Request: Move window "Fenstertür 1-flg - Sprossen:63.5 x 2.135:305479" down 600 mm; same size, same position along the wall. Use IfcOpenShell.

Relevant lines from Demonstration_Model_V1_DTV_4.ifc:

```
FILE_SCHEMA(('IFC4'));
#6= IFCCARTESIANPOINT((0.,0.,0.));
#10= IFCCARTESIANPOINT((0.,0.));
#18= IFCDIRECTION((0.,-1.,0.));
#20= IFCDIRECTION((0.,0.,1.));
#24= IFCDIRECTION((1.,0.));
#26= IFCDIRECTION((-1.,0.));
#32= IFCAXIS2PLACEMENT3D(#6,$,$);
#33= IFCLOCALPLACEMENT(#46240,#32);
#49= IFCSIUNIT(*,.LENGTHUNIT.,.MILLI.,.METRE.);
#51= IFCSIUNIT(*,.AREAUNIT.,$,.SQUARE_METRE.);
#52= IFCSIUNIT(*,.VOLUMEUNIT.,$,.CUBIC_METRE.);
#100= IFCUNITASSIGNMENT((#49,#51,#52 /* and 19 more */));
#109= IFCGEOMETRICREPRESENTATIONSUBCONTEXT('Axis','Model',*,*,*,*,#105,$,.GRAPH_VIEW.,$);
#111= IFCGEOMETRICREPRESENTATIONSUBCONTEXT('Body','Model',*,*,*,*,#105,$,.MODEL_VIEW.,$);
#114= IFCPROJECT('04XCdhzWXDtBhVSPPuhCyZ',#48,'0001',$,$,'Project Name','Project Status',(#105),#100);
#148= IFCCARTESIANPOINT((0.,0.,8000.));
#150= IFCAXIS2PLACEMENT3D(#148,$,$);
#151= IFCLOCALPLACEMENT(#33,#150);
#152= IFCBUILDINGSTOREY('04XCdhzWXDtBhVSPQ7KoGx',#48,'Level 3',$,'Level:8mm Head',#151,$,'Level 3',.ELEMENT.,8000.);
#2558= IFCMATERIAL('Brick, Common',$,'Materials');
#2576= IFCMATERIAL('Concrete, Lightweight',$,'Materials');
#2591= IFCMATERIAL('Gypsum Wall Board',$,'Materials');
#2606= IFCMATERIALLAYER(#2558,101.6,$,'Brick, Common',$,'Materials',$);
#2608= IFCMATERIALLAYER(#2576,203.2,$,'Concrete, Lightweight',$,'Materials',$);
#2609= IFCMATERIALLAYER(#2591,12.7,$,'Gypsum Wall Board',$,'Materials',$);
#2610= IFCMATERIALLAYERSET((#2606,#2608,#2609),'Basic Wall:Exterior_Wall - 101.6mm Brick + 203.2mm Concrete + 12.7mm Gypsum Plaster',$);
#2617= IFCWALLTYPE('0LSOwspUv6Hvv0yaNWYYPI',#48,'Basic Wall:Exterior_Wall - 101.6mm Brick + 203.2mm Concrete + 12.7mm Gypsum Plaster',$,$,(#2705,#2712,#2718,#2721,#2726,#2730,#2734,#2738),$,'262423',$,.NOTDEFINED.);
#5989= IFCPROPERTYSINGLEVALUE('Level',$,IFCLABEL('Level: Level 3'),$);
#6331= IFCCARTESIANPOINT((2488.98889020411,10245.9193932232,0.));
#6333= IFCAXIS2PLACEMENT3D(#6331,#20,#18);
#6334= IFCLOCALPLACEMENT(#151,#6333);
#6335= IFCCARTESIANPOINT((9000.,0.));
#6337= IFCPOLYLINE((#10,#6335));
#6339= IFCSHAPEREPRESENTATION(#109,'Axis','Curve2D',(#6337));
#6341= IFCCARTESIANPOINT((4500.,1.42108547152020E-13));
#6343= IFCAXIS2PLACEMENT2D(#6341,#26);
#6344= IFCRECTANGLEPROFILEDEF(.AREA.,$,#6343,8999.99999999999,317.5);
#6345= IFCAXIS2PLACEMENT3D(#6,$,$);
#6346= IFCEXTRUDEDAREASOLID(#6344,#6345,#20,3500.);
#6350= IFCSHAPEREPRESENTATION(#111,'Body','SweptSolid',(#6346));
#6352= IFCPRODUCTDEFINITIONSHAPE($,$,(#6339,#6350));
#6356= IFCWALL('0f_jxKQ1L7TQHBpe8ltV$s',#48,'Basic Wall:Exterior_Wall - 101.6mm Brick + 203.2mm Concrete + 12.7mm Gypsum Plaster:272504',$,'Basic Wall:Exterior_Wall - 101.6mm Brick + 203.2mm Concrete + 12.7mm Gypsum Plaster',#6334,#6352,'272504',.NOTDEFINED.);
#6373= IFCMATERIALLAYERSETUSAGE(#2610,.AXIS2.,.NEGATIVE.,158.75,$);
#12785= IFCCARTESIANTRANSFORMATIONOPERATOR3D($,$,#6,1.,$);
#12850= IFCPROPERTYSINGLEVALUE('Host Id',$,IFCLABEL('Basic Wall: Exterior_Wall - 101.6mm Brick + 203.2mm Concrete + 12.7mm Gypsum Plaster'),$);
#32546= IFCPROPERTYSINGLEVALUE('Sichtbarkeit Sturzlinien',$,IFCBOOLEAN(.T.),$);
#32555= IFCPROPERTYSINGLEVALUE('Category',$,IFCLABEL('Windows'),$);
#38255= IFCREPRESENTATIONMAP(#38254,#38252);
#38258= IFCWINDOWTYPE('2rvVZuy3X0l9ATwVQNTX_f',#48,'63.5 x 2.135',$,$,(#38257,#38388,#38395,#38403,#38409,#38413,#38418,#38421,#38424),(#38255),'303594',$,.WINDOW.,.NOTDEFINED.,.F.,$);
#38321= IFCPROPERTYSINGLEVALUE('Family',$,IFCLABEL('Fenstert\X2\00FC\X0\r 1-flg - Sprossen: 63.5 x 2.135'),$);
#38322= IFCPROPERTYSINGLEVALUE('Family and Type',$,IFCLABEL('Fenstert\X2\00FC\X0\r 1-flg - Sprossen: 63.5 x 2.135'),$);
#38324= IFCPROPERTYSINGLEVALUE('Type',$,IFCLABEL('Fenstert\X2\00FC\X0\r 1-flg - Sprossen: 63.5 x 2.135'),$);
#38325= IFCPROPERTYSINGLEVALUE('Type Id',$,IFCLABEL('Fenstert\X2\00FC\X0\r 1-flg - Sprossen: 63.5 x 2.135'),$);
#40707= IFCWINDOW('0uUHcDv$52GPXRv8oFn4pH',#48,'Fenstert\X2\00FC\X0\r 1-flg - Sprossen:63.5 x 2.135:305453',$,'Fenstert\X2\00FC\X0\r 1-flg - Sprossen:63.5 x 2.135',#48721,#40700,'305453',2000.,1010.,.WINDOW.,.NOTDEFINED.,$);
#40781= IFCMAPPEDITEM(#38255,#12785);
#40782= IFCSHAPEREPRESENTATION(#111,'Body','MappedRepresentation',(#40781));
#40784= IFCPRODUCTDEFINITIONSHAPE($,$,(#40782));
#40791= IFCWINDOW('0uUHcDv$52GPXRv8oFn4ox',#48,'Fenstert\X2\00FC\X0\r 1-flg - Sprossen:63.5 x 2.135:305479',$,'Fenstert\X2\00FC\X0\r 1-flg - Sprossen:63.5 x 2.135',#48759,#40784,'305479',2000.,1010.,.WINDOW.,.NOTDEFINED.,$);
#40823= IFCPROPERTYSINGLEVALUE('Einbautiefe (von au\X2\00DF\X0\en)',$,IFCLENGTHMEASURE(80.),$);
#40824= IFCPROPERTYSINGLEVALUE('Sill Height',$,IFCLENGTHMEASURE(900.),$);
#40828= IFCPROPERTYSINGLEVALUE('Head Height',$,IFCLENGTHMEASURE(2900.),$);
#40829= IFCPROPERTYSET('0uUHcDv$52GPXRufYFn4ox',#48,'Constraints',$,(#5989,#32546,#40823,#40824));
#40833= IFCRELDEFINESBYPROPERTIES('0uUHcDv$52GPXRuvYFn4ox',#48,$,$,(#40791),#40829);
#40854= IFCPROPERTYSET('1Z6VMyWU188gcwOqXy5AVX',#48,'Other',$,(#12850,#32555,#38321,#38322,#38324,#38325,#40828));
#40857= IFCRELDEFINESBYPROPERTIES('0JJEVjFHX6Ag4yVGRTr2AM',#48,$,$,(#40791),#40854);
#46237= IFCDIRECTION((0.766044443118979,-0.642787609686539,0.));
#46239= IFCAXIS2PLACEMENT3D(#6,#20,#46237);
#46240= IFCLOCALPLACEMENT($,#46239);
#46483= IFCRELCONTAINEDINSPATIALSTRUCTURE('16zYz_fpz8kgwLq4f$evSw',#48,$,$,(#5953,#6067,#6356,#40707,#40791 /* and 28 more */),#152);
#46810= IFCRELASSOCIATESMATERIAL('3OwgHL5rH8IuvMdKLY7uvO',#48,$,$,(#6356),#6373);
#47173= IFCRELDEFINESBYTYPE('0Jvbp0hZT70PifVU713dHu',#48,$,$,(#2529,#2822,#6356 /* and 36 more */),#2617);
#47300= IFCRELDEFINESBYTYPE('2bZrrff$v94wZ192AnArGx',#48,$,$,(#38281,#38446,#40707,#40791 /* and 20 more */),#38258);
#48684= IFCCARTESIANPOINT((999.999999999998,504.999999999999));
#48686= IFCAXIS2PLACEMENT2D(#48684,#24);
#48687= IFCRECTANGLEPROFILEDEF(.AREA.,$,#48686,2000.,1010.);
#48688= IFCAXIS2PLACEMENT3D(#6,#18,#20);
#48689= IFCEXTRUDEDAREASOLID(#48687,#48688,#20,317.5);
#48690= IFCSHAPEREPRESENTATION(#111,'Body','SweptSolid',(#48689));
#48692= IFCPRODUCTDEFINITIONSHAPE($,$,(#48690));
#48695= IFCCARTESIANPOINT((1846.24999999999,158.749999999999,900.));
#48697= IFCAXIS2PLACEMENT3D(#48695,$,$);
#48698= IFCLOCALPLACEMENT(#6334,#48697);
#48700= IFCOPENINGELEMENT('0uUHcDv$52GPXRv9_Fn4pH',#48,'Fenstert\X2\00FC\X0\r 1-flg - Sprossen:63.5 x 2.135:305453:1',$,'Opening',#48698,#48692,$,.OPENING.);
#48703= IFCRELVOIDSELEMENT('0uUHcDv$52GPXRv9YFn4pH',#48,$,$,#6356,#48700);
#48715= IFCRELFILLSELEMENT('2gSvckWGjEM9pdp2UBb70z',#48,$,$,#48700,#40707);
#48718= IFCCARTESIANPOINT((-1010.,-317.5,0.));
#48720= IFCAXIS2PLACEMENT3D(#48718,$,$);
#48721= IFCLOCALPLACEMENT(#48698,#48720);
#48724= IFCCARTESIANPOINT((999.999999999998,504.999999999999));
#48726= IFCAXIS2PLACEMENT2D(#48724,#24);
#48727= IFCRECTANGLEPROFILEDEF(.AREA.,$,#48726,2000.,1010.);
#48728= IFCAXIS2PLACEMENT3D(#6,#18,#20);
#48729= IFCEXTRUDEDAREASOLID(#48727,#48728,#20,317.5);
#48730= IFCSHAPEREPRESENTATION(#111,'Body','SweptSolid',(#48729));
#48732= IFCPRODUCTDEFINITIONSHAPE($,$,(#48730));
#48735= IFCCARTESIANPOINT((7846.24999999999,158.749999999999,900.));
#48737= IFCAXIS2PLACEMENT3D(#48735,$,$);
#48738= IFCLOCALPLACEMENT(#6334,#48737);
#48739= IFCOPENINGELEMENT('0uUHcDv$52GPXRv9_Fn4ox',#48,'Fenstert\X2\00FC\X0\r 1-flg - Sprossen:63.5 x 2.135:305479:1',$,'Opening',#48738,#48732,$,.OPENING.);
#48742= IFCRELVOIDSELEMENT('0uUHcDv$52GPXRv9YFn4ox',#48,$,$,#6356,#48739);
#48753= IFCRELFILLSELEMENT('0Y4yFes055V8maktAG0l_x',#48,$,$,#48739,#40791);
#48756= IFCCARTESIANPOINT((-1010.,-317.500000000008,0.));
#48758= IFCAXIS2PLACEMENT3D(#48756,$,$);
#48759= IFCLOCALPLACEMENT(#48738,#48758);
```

```python
import numpy as np
import ifcopenshell
import ifcopenshell.api.geometry
import ifcopenshell.api.pset
import ifcopenshell.util.element
import ifcopenshell.util.placement
import ifcopenshell.util.unit

model = ifcopenshell.open("Demonstration_Model_V1_DTV_4.ifc")
unit_scale = ifcopenshell.util.unit.calculate_unit_scale(model)

window = model.by_guid("0uUHcDv$52GPXRv8oFn4ox")
opening = window.FillsVoids[0].RelatingOpeningElement
dz = -0.6 / unit_scale

shift = np.array([0.0, 0.0, dz])
# The window is placed relative to its opening, so it follows when the opening moves.
matrix = ifcopenshell.util.placement.get_local_placement(opening.ObjectPlacement)
matrix[:3, 3] += shift
ifcopenshell.api.geometry.edit_object_placement(
    model, product=opening, matrix=matrix, is_si=False, should_transform_children=True
)

# Keep the stored heights in step.
pset = model.by_id(ifcopenshell.util.element.get_pset(window, "Constraints", should_inherit=False)["id"])
ifcopenshell.api.pset.edit_pset(model, pset=pset, properties={
    "Sill Height": model.create_entity("IfcLengthMeasure", ifcopenshell.util.element.get_pset(window, "Constraints", "Sill Height") + dz),
})
pset = model.by_id(ifcopenshell.util.element.get_pset(window, "Other", should_inherit=False)["id"])
ifcopenshell.api.pset.edit_pset(model, pset=pset, properties={
    "Head Height": model.create_entity("IfcLengthMeasure", ifcopenshell.util.element.get_pset(window, "Other", "Head Height") + dz),
})

print(f"moved by {dz * unit_scale:+.3f} m")

model.write("Demonstration_Model_V1_DTV_4_v2.ifc")
```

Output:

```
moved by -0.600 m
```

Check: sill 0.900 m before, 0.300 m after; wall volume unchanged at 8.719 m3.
